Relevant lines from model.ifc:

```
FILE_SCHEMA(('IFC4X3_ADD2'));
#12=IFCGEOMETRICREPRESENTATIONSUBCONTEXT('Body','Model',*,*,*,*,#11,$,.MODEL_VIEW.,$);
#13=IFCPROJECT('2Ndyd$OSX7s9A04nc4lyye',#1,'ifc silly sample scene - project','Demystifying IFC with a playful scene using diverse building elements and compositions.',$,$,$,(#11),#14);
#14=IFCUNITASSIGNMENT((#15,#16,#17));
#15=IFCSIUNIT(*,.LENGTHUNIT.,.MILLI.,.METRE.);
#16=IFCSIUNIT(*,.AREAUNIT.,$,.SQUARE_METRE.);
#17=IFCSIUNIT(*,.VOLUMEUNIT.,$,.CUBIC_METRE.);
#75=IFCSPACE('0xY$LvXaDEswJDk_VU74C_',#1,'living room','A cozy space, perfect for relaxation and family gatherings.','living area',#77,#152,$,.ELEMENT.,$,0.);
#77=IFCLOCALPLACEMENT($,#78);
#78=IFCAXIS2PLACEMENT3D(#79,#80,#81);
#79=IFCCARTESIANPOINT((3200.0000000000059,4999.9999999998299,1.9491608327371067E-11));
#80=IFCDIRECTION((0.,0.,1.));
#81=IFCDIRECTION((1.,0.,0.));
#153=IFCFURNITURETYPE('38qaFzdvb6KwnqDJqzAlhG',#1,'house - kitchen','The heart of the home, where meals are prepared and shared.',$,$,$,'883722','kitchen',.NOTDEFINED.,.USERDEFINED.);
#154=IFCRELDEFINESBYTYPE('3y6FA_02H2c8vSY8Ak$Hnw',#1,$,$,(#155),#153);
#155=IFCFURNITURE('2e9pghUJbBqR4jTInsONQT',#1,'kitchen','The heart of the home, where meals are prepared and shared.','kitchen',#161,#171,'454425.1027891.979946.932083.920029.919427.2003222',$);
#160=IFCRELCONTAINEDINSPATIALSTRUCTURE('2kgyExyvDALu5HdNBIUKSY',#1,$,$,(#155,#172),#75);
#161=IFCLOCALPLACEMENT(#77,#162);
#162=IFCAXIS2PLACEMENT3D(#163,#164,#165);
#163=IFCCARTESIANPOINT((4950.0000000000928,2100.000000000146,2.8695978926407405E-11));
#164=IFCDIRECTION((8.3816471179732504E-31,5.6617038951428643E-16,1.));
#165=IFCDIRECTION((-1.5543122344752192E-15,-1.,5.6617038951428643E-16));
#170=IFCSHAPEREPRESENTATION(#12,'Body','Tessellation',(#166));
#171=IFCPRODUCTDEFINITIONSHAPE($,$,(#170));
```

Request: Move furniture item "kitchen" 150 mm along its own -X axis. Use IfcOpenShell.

```python
import ifcopenshell
import ifcopenshell.api.geometry
import ifcopenshell.util.placement

model = ifcopenshell.open("model.ifc")

item = model.by_id(155)
matrix = ifcopenshell.util.placement.get_local_placement(item.ObjectPlacement)
matrix[:3, 3] -= matrix[:3, 0] * 150.0
ifcopenshell.api.geometry.edit_object_placement(model, product=item, matrix=matrix, is_si=False)

print(ifcopenshell.util.placement.get_local_placement(item.ObjectPlacement).round(3) + 0.0)

model.write("model_edited.ifc")
```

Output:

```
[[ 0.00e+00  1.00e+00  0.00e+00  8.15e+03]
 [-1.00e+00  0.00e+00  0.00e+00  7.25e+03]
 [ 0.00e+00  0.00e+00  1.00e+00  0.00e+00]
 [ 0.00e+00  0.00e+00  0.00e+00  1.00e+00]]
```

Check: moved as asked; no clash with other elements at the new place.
